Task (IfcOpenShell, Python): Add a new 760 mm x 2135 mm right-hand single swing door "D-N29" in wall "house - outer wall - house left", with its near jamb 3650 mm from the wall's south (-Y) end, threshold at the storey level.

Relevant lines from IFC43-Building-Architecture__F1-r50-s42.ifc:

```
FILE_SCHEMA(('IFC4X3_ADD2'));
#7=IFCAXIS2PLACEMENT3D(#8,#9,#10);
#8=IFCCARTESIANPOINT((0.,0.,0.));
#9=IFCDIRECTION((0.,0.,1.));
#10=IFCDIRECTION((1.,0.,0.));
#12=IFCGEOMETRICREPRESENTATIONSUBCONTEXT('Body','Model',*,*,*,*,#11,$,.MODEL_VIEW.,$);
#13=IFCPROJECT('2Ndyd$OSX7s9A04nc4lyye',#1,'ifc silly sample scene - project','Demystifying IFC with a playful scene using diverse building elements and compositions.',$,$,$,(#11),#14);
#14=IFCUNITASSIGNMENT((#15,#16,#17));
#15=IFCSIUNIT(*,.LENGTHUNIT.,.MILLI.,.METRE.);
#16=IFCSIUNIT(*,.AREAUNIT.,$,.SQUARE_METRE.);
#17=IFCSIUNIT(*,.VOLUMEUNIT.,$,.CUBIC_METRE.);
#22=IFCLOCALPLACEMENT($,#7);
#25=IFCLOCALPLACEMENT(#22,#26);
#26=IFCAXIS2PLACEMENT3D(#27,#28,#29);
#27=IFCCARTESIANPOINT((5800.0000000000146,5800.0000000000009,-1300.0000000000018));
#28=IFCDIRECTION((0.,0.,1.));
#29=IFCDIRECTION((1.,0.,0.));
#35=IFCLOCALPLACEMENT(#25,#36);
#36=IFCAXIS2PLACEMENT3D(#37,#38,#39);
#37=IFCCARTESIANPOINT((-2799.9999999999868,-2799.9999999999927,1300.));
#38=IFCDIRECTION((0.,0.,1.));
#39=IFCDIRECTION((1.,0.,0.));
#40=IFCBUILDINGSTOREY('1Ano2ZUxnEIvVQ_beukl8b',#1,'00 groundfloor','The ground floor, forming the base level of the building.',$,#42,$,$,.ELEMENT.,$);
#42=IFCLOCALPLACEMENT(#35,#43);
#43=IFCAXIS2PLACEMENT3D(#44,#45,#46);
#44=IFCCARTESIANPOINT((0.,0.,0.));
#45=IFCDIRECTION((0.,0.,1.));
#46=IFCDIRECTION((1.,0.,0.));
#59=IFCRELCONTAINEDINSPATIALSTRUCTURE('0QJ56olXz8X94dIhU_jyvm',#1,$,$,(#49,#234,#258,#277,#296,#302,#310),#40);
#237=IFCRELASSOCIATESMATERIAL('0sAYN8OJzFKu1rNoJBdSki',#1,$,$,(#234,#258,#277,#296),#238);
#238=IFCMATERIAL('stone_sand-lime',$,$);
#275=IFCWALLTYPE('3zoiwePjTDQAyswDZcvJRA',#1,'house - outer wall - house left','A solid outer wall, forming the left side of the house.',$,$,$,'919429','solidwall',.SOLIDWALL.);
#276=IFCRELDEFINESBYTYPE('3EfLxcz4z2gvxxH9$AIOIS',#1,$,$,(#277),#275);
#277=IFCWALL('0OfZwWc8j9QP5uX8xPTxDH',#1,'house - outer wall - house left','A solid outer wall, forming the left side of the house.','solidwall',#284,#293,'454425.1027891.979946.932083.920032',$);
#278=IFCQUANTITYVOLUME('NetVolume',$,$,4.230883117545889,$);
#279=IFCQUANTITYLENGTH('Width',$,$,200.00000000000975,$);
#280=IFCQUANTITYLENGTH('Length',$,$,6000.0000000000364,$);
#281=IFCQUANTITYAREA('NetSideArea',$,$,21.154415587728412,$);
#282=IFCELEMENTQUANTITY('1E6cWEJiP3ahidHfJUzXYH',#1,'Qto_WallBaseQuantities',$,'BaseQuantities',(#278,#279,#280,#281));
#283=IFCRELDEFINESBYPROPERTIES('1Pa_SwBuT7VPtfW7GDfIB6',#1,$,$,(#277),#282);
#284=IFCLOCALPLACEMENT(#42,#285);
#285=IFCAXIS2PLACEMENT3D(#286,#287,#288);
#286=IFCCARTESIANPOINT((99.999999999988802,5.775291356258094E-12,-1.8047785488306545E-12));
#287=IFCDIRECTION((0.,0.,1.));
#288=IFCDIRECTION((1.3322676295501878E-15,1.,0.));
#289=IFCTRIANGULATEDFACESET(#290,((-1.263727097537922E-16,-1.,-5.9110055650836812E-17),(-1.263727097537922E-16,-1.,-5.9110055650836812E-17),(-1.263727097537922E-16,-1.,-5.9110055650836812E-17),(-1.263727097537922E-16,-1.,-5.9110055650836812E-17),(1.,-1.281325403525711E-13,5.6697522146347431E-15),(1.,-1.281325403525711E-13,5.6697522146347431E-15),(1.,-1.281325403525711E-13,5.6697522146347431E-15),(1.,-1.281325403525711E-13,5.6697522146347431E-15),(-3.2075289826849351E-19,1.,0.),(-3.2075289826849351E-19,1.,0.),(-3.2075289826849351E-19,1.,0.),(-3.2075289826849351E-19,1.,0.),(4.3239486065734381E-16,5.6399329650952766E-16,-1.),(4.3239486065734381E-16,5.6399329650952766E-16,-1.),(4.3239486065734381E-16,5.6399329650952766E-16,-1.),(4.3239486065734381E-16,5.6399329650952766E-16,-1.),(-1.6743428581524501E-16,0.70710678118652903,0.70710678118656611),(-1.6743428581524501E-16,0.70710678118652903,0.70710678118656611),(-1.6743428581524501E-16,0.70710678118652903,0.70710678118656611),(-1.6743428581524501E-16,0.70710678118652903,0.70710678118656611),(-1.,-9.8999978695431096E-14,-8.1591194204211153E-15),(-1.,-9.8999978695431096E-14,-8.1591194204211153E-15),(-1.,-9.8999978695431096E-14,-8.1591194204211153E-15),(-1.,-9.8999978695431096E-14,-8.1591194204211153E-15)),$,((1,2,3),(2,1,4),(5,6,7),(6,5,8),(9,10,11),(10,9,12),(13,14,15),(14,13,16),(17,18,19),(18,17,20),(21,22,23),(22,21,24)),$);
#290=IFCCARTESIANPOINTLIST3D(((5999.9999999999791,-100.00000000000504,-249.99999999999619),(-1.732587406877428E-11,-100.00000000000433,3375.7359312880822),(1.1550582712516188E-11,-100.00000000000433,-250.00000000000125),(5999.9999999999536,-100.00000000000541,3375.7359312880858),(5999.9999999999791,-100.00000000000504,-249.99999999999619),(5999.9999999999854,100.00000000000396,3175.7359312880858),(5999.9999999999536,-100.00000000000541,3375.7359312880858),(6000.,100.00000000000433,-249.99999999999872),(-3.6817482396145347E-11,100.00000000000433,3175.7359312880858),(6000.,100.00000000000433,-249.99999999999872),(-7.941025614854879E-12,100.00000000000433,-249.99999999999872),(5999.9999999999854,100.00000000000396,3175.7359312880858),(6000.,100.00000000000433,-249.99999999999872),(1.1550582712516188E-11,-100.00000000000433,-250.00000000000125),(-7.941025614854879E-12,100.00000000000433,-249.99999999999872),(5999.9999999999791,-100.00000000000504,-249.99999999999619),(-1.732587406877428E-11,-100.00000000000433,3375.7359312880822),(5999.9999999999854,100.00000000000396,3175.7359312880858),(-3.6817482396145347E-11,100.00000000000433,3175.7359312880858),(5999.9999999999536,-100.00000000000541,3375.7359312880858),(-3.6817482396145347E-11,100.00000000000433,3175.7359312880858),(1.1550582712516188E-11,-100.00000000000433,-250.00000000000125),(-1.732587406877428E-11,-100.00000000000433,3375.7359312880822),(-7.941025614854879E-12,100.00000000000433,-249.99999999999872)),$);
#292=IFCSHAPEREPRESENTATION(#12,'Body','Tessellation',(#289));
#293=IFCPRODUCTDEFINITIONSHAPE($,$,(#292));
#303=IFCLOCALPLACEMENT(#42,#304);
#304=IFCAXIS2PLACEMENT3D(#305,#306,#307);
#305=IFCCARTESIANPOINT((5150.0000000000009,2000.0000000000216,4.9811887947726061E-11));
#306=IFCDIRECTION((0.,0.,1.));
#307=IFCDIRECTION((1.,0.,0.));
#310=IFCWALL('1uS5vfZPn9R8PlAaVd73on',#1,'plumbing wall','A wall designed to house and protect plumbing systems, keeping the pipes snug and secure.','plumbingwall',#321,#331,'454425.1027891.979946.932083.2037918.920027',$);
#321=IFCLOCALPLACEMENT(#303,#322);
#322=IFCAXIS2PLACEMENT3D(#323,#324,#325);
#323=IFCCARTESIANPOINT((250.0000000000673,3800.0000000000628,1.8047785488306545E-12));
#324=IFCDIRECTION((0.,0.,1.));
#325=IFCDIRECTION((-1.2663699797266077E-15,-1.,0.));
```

```python
import numpy as np
import ifcopenshell
import ifcopenshell.api.feature
import ifcopenshell.api.geometry
import ifcopenshell.api.pset
import ifcopenshell.api.root
import ifcopenshell.api.spatial
import ifcopenshell.geom
import ifcopenshell.util.element
import ifcopenshell.util.placement
import ifcopenshell.util.representation
import ifcopenshell.util.shape
import ifcopenshell.util.unit

model = ifcopenshell.open("IFC43-Building-Architecture__F1-r50-s42.ifc")
unit_scale = ifcopenshell.util.unit.calculate_unit_scale(model)
area_scale = ifcopenshell.util.unit.calculate_unit_scale(model, "AREAUNIT")
volume_scale = ifcopenshell.util.unit.calculate_unit_scale(model, "VOLUMEUNIT")
settings = ifcopenshell.geom.settings()


def volume(element):
    """Net volume in cubic metres, openings subtracted."""
    shape = ifcopenshell.geom.create_shape(settings, element)
    return ifcopenshell.util.shape.get_volume(shape.geometry)


wall = model.by_guid("0OfZwWc8j9QP5uX8xPTxDH")
storey = ifcopenshell.util.element.get_container(wall, ifc_class="IfcBuildingStorey")
context = ifcopenshell.util.representation.get_context(model, "Model", "Body", "MODEL_VIEW")
before = volume(wall)

width, height, from_end, sill = 0.76, 2.135, 3.65, 0.0  # metres

# The wall runs along its own X axis, and the end named is its -X end.
wall_shape = ifcopenshell.geom.create_shape(settings, wall)
x, y, z = ifcopenshell.util.shape.get_vertices(wall_shape.geometry).T
start = x.min() + from_end
face, thickness = float(y.min()), float(y.max() - y.min())
wall_matrix = ifcopenshell.util.placement.get_local_placement(wall.ObjectPlacement)
level = ifcopenshell.util.placement.get_local_placement(storey.ObjectPlacement)[2, 3]


def in_wall(x, y):
    """Placement at x, y metres in the wall's axes, at sill height."""
    matrix = wall_matrix.copy()
    matrix[:, 3] = wall_matrix @ np.array([x / unit_scale, y / unit_scale, 0.0, 1.0])
    matrix[2, 3] = level + sill / unit_scale
    return matrix


# Opening: a box that overshoots both wall faces by 50 mm.
opening = ifcopenshell.api.root.create_entity(model, ifc_class="IfcOpeningElement", predefined_type="OPENING")
box = ifcopenshell.api.geometry.add_wall_representation(
    model, context=context, length=width, height=height, thickness=thickness + 0.1
)
ifcopenshell.api.geometry.assign_representation(model, product=opening, representation=box)
ifcopenshell.api.geometry.edit_object_placement(model, product=opening, matrix=in_wall(start, face - 0.05), is_si=False)
ifcopenshell.api.feature.add_feature(model, feature=opening, element=wall)

door = ifcopenshell.api.root.create_entity(model, ifc_class="IfcDoor", name="D-N29", predefined_type="DOOR")
door.OverallWidth, door.OverallHeight = width / unit_scale, height / unit_scale
door.OperationType = "SINGLE_SWING_RIGHT"
body = ifcopenshell.api.geometry.add_door_representation(
    model,
    context=context,
    overall_width=door.OverallWidth,
    overall_height=door.OverallHeight,
    operation_type="SINGLE_SWING_RIGHT",
    lining_properties={"LiningDepth": thickness / unit_scale, "ThresholdDepth": thickness / unit_scale},
)
ifcopenshell.api.geometry.assign_representation(model, product=door, representation=body)
ifcopenshell.api.spatial.assign_container(model, products=[door], relating_structure=storey)
ifcopenshell.api.feature.add_filling(model, opening=opening, element=door)

# The lining spans the wall, so the door starts at the wall face.
ifcopenshell.api.geometry.edit_object_placement(model, product=door, matrix=in_wall(start, face), is_si=False)

after = volume(wall)

# Update the wall's stored quantities.
qto = model.by_id(ifcopenshell.util.element.get_pset(wall, "Qto_WallBaseQuantities", should_inherit=False)["id"])
ifcopenshell.api.pset.edit_qto(model, qto=qto, properties={
    "NetVolume": after / volume_scale,
    "NetSideArea": after / thickness / area_scale,
})

print(f"wall volume {before:.3f} -> {after:.3f} m3")

model.write("IFC43-Building-Architecture__F1-r50-s42_v2.ifc")
```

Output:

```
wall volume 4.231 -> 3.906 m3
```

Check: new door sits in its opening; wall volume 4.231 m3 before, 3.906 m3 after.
